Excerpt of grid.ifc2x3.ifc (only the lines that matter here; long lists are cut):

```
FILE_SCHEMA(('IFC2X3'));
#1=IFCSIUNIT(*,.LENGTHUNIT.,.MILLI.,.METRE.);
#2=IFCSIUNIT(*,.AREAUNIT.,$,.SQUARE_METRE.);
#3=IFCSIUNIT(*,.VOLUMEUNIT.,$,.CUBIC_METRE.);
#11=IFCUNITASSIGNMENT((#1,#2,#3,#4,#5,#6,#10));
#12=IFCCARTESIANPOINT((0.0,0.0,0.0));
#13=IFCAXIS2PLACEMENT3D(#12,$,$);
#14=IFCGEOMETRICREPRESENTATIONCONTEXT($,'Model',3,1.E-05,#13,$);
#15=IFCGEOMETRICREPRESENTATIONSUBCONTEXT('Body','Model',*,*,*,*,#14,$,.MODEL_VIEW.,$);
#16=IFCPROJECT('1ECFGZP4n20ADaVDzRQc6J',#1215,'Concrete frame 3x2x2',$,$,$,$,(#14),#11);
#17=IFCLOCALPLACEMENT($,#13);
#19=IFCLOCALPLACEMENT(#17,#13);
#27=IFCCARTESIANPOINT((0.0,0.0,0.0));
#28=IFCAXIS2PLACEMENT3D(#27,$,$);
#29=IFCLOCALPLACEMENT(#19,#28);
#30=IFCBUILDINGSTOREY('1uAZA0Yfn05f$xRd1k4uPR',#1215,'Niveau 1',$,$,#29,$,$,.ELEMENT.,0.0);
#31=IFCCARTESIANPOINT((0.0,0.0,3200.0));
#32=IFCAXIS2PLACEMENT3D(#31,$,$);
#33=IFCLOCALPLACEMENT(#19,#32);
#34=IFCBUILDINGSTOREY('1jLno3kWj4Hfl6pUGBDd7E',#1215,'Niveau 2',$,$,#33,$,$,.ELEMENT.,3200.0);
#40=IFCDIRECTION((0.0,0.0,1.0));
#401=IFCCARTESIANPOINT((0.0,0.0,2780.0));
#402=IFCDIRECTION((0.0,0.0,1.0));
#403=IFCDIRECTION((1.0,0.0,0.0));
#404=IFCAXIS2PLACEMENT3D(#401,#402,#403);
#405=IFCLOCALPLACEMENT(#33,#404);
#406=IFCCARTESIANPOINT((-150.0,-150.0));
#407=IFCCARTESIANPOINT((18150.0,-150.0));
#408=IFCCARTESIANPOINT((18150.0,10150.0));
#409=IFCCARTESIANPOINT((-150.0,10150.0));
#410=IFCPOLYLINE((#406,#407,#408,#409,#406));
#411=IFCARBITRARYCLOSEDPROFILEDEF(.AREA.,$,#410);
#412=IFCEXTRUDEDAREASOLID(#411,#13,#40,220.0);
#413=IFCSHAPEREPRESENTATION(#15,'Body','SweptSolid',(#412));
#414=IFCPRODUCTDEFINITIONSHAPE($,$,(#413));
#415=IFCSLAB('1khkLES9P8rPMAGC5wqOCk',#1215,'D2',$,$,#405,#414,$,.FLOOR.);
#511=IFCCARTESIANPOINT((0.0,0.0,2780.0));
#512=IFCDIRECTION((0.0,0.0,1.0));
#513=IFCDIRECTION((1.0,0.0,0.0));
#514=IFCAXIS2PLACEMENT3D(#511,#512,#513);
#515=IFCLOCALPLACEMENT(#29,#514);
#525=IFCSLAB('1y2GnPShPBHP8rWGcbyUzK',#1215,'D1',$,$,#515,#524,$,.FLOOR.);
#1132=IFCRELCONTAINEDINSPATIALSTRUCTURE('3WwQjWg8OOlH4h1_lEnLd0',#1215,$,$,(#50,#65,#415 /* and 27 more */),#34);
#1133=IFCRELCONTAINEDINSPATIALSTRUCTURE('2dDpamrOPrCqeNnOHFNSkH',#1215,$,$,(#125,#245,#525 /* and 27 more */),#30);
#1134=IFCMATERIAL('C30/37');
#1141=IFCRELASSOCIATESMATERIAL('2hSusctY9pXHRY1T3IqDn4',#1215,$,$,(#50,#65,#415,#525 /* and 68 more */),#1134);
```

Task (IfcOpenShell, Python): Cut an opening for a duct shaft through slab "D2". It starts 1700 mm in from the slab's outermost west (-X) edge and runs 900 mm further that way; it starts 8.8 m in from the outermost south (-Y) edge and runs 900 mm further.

```python
import numpy as np
import ifcopenshell
import ifcopenshell.api.feature
import ifcopenshell.api.geometry
import ifcopenshell.api.root
import ifcopenshell.geom
import ifcopenshell.util.placement
import ifcopenshell.util.representation
import ifcopenshell.util.shape
import ifcopenshell.util.unit

model = ifcopenshell.open("grid.ifc2x3.ifc")
unit_scale = ifcopenshell.util.unit.calculate_unit_scale(model)
settings = ifcopenshell.geom.settings()


def volume(element):
    """Net volume in cubic metres, openings subtracted."""
    shape = ifcopenshell.geom.create_shape(settings, element)
    return ifcopenshell.util.shape.get_volume(shape.geometry)


slab = model.by_id(415)
before = volume(slab)

# Extent in the slab's own axes, in metres. The edges named are its -X and -Y sides.
slab_shape = ifcopenshell.geom.create_shape(settings, slab)
vertices = ifcopenshell.util.shape.get_vertices(slab_shape.geometry)
x_min, y_min, bottom = vertices.min(axis=0)
top = vertices[:, 2].max()

opening = ifcopenshell.api.root.create_entity(model, ifc_class="IfcOpeningElement", name="Duct shaft opening")
context = ifcopenshell.util.representation.get_context(model, "Model", "Body", "MODEL_VIEW")
width, depth = 0.9, 0.9
outline = [(0.0, 0.0), (width, 0.0), (width, depth), (0.0, depth), (0.0, 0.0)]
# Overshoot both faces by 50 mm so the cut is clean.
shape = ifcopenshell.api.geometry.add_slab_representation(
    model, context=context, depth=top - bottom + 0.1, polyline=outline
)
ifcopenshell.api.geometry.assign_representation(model, product=opening, representation=shape)

matrix = ifcopenshell.util.placement.get_local_placement(slab.ObjectPlacement)
matrix[:, 3] = matrix @ np.append(np.array([x_min + 1.7, y_min + 8.8, bottom - 0.05]) / unit_scale, 1.0)
ifcopenshell.api.geometry.edit_object_placement(model, product=opening, matrix=matrix, is_si=False)
ifcopenshell.api.feature.add_feature(model, feature=opening, element=slab)

after = volume(slab)

print(f"slab volume {before:.3f} -> {after:.3f} m3")

model.write("grid.ifc2x3-out.ifc")
```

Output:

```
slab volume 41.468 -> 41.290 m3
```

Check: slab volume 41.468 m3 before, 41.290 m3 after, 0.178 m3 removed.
